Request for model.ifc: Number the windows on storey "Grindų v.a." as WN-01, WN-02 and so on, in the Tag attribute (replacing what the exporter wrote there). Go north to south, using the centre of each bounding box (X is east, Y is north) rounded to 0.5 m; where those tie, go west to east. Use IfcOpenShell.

First a look at what the model holds.

```python
import ifcopenshell
import ifcopenshell.util.element
import ifcopenshell.util.placement

model = ifcopenshell.open("model.ifc")
print(model.schema)
storey = next(s for s in model.by_type("IfcBuildingStorey") if s.Name == "Grindų v.a.")
windows = [e for e in ifcopenshell.util.element.get_decomposition(storey) if e.is_a("IfcWindow")]
for e in sorted(windows, key=lambda e: e.id()):
    origin = ifcopenshell.util.placement.get_local_placement(e.ObjectPlacement)[:3, 3]
    print(e.id(), e.Tag, e.Name, origin.round(2) + 0.0, sep=" | ")
```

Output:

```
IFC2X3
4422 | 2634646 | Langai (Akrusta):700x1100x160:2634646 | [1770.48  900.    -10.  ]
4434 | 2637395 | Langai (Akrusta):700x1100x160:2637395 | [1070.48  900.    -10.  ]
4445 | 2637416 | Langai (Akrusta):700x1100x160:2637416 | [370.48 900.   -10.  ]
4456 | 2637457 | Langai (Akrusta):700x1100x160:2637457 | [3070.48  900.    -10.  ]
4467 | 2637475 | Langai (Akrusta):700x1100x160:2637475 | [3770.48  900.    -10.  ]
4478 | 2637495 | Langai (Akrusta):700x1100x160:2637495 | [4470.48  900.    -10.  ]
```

```python
import ifcopenshell
import ifcopenshell.geom
import ifcopenshell.util.element
import ifcopenshell.util.shape

model = ifcopenshell.open("model.ifc")
settings = ifcopenshell.geom.settings()
settings.set("use-world-coords", True)


def centre(element):
    shape = ifcopenshell.geom.create_shape(settings, element)
    return ifcopenshell.util.shape.get_bbox_centroid(shape.geometry)


storey = next(s for s in model.by_type("IfcBuildingStorey") if s.Name == "Grindų v.a.")
windows = [e for e in ifcopenshell.util.element.get_decomposition(storey) if e.is_a("IfcWindow")]

# Insertion points can sit at a corner or the storey origin, so sort by the geometry (in metres).
centres = {e: centre(e) for e in windows}
windows.sort(key=lambda e: (-round(centres[e][1] / 0.5), centres[e][0]))

for i, e in enumerate(windows, start=1):
    number = f"WN-{i:02d}"
    e.Tag = number
    print(e.id(), number)

model.write("model_rev.ifc")
```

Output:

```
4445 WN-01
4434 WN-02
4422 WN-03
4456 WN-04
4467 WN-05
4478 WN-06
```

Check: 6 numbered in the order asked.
